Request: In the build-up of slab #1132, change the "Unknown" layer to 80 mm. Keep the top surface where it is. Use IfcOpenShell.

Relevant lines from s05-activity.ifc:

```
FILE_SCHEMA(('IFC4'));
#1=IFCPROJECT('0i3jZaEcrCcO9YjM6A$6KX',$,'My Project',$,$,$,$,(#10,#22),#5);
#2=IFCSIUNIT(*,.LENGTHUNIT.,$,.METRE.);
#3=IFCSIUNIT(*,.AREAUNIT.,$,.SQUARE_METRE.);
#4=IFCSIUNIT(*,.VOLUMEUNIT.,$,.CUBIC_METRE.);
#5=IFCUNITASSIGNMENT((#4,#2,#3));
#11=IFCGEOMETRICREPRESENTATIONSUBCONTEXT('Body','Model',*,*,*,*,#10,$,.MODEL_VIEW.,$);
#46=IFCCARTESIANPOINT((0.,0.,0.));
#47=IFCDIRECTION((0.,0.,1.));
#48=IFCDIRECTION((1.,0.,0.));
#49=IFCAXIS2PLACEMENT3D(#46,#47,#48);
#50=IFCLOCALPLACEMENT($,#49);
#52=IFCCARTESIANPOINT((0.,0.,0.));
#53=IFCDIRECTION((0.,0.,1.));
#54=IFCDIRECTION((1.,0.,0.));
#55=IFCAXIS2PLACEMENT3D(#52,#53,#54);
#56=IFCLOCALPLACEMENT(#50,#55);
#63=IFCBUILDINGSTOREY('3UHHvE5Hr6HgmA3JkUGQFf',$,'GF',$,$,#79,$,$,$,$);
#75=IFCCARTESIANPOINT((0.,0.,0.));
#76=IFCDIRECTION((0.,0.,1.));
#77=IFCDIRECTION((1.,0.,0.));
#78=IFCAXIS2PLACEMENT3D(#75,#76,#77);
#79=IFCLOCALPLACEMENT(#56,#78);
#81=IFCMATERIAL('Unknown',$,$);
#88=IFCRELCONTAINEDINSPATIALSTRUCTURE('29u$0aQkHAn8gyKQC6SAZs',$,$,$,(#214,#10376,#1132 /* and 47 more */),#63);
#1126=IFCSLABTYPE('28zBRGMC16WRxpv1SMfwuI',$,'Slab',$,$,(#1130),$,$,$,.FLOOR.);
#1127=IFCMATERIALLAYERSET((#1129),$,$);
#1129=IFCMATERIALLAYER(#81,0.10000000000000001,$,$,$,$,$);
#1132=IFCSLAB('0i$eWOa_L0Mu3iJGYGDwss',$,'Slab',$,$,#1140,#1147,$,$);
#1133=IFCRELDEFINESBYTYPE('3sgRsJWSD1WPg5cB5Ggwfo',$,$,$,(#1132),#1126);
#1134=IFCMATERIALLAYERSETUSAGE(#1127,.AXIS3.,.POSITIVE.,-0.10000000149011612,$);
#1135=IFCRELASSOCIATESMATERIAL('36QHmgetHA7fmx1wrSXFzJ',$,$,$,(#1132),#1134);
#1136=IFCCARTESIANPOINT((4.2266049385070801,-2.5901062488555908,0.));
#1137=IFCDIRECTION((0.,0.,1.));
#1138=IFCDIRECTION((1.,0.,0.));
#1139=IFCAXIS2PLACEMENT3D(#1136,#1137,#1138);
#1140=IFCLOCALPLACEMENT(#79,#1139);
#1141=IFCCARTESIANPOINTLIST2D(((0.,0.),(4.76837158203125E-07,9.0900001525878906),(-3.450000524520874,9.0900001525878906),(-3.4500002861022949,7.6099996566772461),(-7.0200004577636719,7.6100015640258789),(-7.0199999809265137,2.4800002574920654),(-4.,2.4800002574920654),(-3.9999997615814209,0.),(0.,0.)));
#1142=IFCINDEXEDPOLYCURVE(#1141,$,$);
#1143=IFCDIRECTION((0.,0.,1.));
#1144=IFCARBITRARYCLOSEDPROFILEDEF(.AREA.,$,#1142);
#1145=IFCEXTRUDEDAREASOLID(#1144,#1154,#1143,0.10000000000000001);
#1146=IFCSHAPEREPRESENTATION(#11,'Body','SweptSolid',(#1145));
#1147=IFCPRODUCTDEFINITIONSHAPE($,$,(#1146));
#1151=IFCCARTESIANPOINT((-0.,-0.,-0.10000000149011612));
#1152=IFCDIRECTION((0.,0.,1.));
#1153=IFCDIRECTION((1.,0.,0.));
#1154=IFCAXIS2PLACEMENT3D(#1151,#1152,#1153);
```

```python
import ifcopenshell
import ifcopenshell.util.element
import ifcopenshell.util.representation
import ifcopenshell.util.unit

model = ifcopenshell.open("s05-activity.ifc")
unit_scale = ifcopenshell.util.unit.calculate_unit_scale(model)

layer_set = model.by_id(1127)
layer = next(l for l in layer_set.MaterialLayers if l.Material and l.Material.Name == "Unknown")
change = 0.08 / unit_scale - layer.LayerThickness
layer.LayerThickness += change

# Geometry does not follow the layer set by itself.
slabs = [e for e in ifcopenshell.util.element.get_elements_by_material(model, layer_set) if e.is_a("IfcSlab")]
for slab in sorted(slabs, key=lambda e: e.id()):
    body = ifcopenshell.util.representation.get_representation(slab, "Model", "Body")
    solid = body.Items[0]
    old_depth = solid.Depth
    solid.Depth += change
    # Extruded upwards: lower the start of the extrusion so the top stays.
    x, y, z = solid.Position.Location.Coordinates
    solid.Position.Location = model.createIfcCartesianPoint((x, y, z - change))
    print(slab.id(), f"{old_depth:g} -> {solid.Depth:g}")

# The layers are counted up from the underside, which has moved.
for usage in {ifcopenshell.util.element.get_material(slab) for slab in slabs}:
    usage.OffsetFromReferenceLine -= change

model.write("s05-activity-out.ifc")
```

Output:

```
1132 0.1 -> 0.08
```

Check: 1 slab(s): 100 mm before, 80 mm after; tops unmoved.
